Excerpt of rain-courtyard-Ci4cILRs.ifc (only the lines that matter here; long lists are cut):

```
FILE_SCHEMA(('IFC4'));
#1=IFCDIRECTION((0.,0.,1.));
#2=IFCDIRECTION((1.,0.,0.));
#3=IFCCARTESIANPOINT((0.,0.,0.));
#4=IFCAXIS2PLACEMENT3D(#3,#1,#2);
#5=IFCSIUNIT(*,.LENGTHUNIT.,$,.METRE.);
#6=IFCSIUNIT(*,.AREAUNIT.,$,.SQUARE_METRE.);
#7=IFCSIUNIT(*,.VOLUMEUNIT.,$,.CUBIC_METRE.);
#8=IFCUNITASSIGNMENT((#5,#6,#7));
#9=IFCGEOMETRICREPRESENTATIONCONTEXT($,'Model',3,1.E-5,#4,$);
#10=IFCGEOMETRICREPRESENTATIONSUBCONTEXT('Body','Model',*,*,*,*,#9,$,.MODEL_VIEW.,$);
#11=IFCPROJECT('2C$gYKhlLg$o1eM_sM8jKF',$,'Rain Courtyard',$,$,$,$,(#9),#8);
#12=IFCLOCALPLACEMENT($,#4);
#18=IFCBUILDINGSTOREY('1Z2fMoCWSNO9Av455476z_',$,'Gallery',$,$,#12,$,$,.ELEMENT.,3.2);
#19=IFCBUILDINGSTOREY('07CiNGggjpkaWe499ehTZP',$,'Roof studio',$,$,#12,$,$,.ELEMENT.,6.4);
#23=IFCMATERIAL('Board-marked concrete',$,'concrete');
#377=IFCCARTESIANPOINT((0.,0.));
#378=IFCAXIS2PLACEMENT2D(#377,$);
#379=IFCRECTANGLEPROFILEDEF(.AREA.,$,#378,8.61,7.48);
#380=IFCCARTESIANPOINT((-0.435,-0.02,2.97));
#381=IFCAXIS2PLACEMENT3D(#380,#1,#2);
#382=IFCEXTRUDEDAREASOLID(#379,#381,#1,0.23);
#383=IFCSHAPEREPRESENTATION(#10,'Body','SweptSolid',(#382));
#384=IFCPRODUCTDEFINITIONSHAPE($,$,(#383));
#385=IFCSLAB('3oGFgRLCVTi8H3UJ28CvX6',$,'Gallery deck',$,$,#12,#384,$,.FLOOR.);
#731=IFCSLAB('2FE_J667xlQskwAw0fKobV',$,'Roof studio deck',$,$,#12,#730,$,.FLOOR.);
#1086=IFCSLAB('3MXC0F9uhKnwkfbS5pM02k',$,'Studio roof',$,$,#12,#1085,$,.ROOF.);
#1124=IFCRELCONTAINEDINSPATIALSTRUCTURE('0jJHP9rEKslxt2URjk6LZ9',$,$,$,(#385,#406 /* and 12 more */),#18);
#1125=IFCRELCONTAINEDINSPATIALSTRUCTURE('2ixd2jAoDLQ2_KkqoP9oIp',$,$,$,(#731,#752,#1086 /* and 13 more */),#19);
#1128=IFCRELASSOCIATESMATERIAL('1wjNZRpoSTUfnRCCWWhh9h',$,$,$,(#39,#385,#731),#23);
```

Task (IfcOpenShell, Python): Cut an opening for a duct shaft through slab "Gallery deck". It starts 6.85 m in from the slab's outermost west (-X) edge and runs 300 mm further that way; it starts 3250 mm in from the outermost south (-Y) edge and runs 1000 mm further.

```python
import numpy as np
import ifcopenshell
import ifcopenshell.api.feature
import ifcopenshell.api.geometry
import ifcopenshell.api.root
import ifcopenshell.geom
import ifcopenshell.util.placement
import ifcopenshell.util.representation
import ifcopenshell.util.shape
import ifcopenshell.util.unit

model = ifcopenshell.open("rain-courtyard-Ci4cILRs.ifc")
unit_scale = ifcopenshell.util.unit.calculate_unit_scale(model)
settings = ifcopenshell.geom.settings()


def volume(element):
    """Net volume in cubic metres, openings subtracted."""
    shape = ifcopenshell.geom.create_shape(settings, element)
    return ifcopenshell.util.shape.get_volume(shape.geometry)


slab = model.by_guid("3oGFgRLCVTi8H3UJ28CvX6")
before = volume(slab)

# Extent in the slab's own axes, in metres. The edges named are its -X and -Y sides.
slab_shape = ifcopenshell.geom.create_shape(settings, slab)
vertices = ifcopenshell.util.shape.get_vertices(slab_shape.geometry)
x_min, y_min, bottom = vertices.min(axis=0)
top = vertices[:, 2].max()

opening = ifcopenshell.api.root.create_entity(model, ifc_class="IfcOpeningElement", name="Duct shaft opening", predefined_type="OPENING")
context = ifcopenshell.util.representation.get_context(model, "Model", "Body", "MODEL_VIEW")
width, depth = 0.3, 1
outline = [(0.0, 0.0), (width, 0.0), (width, depth), (0.0, depth), (0.0, 0.0)]
# Overshoot both faces by 50 mm so the cut is clean.
shape = ifcopenshell.api.geometry.add_slab_representation(
    model, context=context, depth=top - bottom + 0.1, polyline=outline
)
ifcopenshell.api.geometry.assign_representation(model, product=opening, representation=shape)

matrix = ifcopenshell.util.placement.get_local_placement(slab.ObjectPlacement)
matrix[:, 3] = matrix @ np.append(np.array([x_min + 6.85, y_min + 3.25, bottom - 0.05]) / unit_scale, 1.0)
ifcopenshell.api.geometry.edit_object_placement(model, product=opening, matrix=matrix, is_si=False)
ifcopenshell.api.feature.add_feature(model, feature=opening, element=slab)

after = volume(slab)

print(f"slab volume {before:.3f} -> {after:.3f} m3")

model.write("rain-courtyard-Ci4cILRs_rev.ifc")
```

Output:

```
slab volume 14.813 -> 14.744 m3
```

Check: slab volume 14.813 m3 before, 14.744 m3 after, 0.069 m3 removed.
